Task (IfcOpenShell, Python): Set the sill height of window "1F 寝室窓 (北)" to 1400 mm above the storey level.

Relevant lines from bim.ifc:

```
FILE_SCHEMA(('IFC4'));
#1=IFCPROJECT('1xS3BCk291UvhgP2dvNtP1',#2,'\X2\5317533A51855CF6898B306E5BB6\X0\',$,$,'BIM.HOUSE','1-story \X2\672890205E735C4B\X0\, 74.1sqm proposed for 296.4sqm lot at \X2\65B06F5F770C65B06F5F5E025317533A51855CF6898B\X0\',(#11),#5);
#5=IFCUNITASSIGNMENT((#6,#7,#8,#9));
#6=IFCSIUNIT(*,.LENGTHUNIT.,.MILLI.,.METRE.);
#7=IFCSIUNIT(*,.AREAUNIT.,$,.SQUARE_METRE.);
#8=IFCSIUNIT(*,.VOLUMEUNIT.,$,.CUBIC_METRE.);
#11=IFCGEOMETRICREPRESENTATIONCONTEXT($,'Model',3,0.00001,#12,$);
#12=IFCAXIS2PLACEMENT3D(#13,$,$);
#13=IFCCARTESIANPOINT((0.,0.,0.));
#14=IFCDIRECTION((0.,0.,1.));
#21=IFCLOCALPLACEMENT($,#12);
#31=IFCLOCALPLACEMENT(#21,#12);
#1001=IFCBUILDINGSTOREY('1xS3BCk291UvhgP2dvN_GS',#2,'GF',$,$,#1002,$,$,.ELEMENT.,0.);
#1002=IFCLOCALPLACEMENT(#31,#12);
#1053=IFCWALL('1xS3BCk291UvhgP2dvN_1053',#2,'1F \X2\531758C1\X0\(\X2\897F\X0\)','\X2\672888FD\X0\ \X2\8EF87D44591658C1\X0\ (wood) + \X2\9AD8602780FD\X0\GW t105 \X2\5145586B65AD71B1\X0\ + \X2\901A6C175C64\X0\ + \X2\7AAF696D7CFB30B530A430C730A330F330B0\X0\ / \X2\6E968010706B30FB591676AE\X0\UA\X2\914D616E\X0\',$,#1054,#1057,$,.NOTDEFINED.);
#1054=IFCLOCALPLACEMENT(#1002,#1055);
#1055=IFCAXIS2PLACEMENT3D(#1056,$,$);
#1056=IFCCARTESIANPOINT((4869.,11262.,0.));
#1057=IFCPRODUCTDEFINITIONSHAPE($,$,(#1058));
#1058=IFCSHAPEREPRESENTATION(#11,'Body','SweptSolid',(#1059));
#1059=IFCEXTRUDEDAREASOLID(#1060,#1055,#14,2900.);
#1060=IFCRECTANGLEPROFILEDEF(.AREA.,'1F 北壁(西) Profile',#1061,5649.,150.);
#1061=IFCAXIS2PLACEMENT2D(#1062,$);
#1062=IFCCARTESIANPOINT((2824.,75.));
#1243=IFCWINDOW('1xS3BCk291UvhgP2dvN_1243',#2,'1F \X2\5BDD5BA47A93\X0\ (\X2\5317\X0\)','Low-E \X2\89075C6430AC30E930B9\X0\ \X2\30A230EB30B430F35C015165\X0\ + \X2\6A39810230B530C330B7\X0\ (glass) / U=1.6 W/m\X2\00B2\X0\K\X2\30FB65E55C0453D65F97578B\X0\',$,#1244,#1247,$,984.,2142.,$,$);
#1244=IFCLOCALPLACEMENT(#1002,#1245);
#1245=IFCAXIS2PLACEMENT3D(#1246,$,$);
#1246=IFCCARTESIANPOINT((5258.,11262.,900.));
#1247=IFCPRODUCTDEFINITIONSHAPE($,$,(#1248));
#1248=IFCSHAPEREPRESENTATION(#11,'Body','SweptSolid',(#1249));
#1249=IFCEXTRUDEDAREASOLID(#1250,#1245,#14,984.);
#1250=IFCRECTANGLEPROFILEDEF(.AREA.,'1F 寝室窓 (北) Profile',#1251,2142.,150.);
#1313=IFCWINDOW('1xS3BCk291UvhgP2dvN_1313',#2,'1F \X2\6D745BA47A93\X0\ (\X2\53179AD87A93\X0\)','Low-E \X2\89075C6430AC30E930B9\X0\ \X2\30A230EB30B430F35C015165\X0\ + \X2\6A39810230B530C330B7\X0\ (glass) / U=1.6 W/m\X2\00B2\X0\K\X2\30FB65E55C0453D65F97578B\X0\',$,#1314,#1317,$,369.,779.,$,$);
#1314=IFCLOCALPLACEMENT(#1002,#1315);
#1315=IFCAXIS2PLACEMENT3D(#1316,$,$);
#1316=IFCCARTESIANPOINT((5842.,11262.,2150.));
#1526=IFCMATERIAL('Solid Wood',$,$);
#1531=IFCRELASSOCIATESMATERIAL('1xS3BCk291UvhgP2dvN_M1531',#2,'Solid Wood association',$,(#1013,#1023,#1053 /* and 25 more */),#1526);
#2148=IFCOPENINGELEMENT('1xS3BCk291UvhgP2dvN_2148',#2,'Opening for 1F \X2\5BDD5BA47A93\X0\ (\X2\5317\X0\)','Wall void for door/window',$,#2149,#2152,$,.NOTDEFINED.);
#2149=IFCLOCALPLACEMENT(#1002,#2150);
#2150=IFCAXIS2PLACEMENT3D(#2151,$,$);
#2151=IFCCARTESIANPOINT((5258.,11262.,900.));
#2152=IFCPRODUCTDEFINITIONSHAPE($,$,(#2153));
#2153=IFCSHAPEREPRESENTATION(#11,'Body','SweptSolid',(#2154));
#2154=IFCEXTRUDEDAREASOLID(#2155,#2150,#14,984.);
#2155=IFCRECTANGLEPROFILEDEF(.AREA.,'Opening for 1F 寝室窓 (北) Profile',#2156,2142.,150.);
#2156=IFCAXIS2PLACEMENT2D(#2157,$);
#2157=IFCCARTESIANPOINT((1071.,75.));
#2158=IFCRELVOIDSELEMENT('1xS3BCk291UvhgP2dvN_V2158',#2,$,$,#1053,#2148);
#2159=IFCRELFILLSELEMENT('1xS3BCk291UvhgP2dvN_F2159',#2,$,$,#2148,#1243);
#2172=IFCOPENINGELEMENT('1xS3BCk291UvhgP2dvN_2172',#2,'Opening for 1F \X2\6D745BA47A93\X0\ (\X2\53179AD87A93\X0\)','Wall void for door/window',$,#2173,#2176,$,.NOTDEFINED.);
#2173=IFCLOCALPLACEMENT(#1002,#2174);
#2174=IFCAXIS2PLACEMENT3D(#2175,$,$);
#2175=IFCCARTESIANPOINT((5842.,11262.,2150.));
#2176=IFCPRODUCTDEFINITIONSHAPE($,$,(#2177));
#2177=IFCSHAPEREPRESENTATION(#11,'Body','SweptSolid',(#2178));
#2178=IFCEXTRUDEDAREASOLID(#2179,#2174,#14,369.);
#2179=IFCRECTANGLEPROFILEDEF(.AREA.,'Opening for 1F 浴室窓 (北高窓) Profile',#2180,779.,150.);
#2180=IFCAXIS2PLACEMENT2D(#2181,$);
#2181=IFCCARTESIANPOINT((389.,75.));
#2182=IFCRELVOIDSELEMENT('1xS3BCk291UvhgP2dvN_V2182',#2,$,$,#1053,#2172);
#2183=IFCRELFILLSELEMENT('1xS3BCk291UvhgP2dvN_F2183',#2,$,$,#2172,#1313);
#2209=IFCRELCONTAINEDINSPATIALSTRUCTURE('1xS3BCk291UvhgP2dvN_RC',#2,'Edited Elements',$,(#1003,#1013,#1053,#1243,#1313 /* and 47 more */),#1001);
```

```python
import numpy as np
import ifcopenshell
import ifcopenshell.api.geometry
import ifcopenshell.geom
import ifcopenshell.util.element
import ifcopenshell.util.placement
import ifcopenshell.util.shape
import ifcopenshell.util.unit

model = ifcopenshell.open("bim.ifc")
unit_scale = ifcopenshell.util.unit.calculate_unit_scale(model)

window = model.by_guid("1xS3BCk291UvhgP2dvN_1243")
opening = window.FillsVoids[0].RelatingOpeningElement
storey = ifcopenshell.util.element.get_container(window, ifc_class="IfcBuildingStorey")
level = ifcopenshell.util.placement.get_local_placement(storey.ObjectPlacement)[2, 3]

# The opening's origin need not be at the sill, so measure its lowest point.
shape = ifcopenshell.geom.create_shape(ifcopenshell.geom.settings(), opening)
bottom = ifcopenshell.util.shape.get_shape_bottom_elevation(shape, shape.geometry) / unit_scale
dz = level + 1.4 / unit_scale - bottom

shift = np.array([0.0, 0.0, dz])
# The window is not placed relative to its opening, so move both.
for product in (opening, window):
    matrix = ifcopenshell.util.placement.get_local_placement(product.ObjectPlacement)
    matrix[:3, 3] += shift
    ifcopenshell.api.geometry.edit_object_placement(model, product=product, matrix=matrix, is_si=False)

print(f"moved by {dz * unit_scale:+.3f} m")

model.write("bim_v2.ifc")
```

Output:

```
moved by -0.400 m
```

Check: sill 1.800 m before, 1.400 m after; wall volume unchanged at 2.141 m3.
